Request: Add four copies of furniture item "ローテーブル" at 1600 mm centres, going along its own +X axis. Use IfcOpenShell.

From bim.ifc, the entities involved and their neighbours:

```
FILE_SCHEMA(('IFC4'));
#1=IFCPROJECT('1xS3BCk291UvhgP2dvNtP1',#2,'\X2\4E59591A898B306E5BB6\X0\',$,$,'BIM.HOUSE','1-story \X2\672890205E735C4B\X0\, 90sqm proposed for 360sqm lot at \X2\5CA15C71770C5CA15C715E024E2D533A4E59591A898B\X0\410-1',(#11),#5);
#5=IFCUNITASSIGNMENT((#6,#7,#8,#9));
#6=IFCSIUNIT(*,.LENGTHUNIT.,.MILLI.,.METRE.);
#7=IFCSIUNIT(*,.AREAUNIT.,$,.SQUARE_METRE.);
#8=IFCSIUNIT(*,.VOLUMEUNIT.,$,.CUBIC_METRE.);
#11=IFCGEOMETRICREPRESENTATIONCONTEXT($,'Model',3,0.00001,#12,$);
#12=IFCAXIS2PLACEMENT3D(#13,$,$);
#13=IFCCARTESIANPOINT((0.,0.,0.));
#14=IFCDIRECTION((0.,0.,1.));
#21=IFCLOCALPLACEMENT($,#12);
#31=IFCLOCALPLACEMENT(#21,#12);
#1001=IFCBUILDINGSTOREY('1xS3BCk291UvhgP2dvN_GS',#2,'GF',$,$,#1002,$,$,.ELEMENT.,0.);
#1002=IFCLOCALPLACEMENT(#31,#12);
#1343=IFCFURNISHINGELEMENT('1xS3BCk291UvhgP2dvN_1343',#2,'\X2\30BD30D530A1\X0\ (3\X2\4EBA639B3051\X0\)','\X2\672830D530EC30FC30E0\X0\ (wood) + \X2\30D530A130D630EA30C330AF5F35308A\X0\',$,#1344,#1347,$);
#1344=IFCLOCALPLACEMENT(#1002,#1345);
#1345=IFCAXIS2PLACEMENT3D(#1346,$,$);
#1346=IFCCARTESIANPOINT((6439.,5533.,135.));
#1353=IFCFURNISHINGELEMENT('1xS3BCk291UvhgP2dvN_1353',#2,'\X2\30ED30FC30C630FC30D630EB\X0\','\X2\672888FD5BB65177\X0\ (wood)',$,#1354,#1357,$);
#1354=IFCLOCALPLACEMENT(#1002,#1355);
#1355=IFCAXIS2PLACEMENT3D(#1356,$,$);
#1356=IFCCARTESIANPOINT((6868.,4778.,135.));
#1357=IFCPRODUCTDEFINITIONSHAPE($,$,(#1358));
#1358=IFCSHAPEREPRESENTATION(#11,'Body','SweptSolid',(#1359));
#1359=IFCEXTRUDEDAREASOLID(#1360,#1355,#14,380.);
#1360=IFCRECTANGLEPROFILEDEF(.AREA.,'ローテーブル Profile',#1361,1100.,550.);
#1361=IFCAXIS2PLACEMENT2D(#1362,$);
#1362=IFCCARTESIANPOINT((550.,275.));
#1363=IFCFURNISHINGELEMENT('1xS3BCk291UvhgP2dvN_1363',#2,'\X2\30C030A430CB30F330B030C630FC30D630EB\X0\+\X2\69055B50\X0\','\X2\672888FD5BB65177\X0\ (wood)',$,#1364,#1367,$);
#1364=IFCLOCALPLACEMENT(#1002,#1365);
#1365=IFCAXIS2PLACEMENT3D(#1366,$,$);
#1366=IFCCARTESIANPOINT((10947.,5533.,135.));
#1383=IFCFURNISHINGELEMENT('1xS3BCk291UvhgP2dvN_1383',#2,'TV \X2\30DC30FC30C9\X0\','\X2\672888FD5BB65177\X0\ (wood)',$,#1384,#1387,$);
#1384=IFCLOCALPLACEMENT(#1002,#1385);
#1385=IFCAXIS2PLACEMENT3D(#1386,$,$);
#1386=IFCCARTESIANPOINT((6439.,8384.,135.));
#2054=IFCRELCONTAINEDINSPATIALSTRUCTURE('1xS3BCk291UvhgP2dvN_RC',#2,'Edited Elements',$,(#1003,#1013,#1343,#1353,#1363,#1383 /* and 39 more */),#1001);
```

```python
import ifcopenshell
import ifcopenshell.api.geometry
import ifcopenshell.api.root
import ifcopenshell.util.element
import ifcopenshell.util.placement
import ifcopenshell.util.unit

model = ifcopenshell.open("bim.ifc")
unit_scale = ifcopenshell.util.unit.calculate_unit_scale(model)


def reuse_history(source, copy):
    """copy_class also copies each property set's owner history, people and application; keep the originals."""
    for rel in copy.IsDefinedBy:
        if rel.is_a("IfcRelDefinesByProperties") and (history := rel.RelatingPropertyDefinition.OwnerHistory):
            rel.RelatingPropertyDefinition.OwnerHistory = source.OwnerHistory
            ifcopenshell.util.element.remove_deep2(model, history)


source = model.by_guid("1xS3BCk291UvhgP2dvN_1353")
base = ifcopenshell.util.placement.get_local_placement(source.ObjectPlacement)
step = base[:3, 0] * 1.6 / unit_scale

for i in range(1, 5):
    copy = ifcopenshell.api.root.copy_class(model, product=source)
    copy.Representation = ifcopenshell.util.element.copy_deep(
        model, source.Representation, exclude=["IfcGeometricRepresentationContext", "IfcRepresentationMap"]
    )
    reuse_history(source, copy)
    matrix = base.copy()
    matrix[:3, 3] += i * step
    print("added at", matrix[:3, 3].round(3) + 0.0)
    ifcopenshell.api.geometry.edit_object_placement(model, product=copy, matrix=matrix, is_si=False)

model.write("bim_rev.ifc")
```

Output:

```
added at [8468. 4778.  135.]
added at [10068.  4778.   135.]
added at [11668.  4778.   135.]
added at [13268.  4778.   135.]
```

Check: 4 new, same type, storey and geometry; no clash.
